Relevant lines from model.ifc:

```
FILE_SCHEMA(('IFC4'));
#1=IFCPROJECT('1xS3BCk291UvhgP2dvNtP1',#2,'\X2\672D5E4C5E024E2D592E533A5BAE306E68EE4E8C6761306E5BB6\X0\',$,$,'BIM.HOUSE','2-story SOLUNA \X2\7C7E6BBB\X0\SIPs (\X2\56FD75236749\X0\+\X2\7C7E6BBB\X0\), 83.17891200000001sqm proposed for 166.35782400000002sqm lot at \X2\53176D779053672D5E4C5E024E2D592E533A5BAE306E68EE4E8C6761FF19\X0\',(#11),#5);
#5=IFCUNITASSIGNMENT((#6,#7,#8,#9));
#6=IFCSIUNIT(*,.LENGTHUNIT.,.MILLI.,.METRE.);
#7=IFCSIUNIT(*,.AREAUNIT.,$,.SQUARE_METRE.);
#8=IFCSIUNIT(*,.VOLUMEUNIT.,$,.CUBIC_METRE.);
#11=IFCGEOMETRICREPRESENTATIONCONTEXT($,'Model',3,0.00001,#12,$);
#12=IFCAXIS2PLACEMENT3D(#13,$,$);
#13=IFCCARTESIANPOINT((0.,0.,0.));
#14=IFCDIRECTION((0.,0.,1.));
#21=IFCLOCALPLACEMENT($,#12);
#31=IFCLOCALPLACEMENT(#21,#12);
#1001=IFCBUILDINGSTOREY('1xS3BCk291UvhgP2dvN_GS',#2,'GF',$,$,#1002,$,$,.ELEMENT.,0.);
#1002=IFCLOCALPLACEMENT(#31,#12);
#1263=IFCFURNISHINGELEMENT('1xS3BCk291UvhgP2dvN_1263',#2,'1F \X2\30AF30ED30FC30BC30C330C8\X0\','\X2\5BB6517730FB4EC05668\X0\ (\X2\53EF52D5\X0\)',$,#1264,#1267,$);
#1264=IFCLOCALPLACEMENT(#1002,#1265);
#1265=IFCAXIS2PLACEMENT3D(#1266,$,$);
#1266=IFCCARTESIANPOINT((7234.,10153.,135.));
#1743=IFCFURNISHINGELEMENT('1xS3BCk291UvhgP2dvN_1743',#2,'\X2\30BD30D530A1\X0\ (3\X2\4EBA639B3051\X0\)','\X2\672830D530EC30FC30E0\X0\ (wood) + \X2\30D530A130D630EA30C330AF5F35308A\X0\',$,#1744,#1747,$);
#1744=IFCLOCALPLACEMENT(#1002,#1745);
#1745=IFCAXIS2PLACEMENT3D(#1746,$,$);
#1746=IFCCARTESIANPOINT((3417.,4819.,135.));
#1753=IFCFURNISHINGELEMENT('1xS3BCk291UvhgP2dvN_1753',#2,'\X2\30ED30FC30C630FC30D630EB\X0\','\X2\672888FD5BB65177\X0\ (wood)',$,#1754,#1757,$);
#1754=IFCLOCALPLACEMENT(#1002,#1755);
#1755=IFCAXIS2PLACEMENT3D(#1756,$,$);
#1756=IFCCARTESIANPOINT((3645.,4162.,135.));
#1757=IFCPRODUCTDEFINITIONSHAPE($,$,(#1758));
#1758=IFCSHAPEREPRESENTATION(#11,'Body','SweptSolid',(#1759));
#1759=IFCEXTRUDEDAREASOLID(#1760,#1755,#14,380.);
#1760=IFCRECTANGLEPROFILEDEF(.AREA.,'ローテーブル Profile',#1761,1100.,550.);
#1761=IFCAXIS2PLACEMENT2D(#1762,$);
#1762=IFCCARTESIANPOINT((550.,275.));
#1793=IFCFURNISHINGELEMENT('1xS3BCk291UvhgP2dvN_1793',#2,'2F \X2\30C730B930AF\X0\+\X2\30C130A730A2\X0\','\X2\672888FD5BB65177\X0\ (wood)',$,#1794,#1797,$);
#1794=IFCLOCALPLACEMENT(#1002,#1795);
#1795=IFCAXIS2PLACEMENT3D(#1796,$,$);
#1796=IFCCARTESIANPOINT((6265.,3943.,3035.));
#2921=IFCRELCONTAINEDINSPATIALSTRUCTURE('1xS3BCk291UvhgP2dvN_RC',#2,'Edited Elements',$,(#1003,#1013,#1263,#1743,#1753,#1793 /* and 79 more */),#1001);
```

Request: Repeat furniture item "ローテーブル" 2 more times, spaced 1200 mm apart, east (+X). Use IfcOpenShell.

```python
import numpy as np
import ifcopenshell
import ifcopenshell.api.geometry
import ifcopenshell.api.root
import ifcopenshell.util.element
import ifcopenshell.util.placement

model = ifcopenshell.open("model.ifc")


def reuse_history(source, copy):
    """copy_class also copies each property set's owner history, people and application; keep the originals."""
    for rel in copy.IsDefinedBy:
        if rel.is_a("IfcRelDefinesByProperties") and (history := rel.RelatingPropertyDefinition.OwnerHistory):
            rel.RelatingPropertyDefinition.OwnerHistory = source.OwnerHistory
            ifcopenshell.util.element.remove_deep2(model, history)


source = model.by_guid("1xS3BCk291UvhgP2dvN_1753")
base = ifcopenshell.util.placement.get_local_placement(source.ObjectPlacement)
step = np.array([1.0, 0.0, 0.0]) * 1200.0

for i in range(1, 3):
    copy = ifcopenshell.api.root.copy_class(model, product=source)
    copy.Representation = ifcopenshell.util.element.copy_deep(
        model, source.Representation, exclude=["IfcGeometricRepresentationContext", "IfcRepresentationMap"]
    )
    reuse_history(source, copy)
    matrix = base.copy()
    matrix[:3, 3] += i * step
    print("added at", matrix[:3, 3].round(3) + 0.0)
    ifcopenshell.api.geometry.edit_object_placement(model, product=copy, matrix=matrix, is_si=False)

model.write("model_v2.ifc")
```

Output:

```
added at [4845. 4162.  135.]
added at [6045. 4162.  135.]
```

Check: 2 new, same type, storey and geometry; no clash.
